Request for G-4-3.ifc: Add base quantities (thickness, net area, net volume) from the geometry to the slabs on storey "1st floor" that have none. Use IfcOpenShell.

First a look at what the model holds.

```python
import ifcopenshell
import ifcopenshell.util.element
import ifcopenshell.util.unit

model = ifcopenshell.open("G-4-3.ifc")
print(model.schema)
for unit_type in ("LENGTHUNIT", "AREAUNIT", "VOLUMEUNIT"):
    print(unit_type, ifcopenshell.util.unit.calculate_unit_scale(model, unit_type))
storey = next(s for s in model.by_type("IfcBuildingStorey") if s.Name == "1st floor")
slabs = [e for e in ifcopenshell.util.element.get_decomposition(storey) if e.is_a("IfcSlab")]
for e in sorted(slabs, key=lambda e: e.id()):
    print(e.id(), e.is_a(), e.Name, list(ifcopenshell.util.element.get_psets(e, qtos_only=True)), sep=" | ")
```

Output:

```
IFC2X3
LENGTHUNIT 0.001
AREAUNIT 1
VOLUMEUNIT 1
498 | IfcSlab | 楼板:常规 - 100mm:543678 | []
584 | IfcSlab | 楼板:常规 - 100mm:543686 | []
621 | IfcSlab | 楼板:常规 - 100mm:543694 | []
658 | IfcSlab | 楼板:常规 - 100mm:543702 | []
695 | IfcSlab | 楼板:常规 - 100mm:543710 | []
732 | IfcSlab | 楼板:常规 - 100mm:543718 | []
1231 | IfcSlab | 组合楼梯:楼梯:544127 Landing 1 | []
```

```python
import ifcopenshell
import ifcopenshell.api.pset
import ifcopenshell.geom
import ifcopenshell.util.element
import ifcopenshell.util.shape
import ifcopenshell.util.unit

model = ifcopenshell.open("G-4-3.ifc")
unit_scale = ifcopenshell.util.unit.calculate_unit_scale(model)
area_scale = ifcopenshell.util.unit.calculate_unit_scale(model, "AREAUNIT")
volume_scale = ifcopenshell.util.unit.calculate_unit_scale(model, "VOLUMEUNIT")
settings = ifcopenshell.geom.settings()

storey = next(s for s in model.by_type("IfcBuildingStorey") if s.Name == "1st floor")
slabs = [e for e in ifcopenshell.util.element.get_decomposition(storey) if e.is_a("IfcSlab")]

for e in sorted(slabs, key=lambda e: e.id()):
    if ifcopenshell.util.element.get_psets(e, qtos_only=True, should_inherit=False):
        continue
    # Geometry comes back in metres, in the element's own axes.
    shape = ifcopenshell.geom.create_shape(settings, e)
    values = {
        "Width": ifcopenshell.util.shape.get_z(shape.geometry) / unit_scale,
        "NetArea": ifcopenshell.util.shape.get_footprint_area(shape.geometry) / area_scale,
        "NetVolume": ifcopenshell.util.shape.get_volume(shape.geometry) / volume_scale,
    }
    qto = ifcopenshell.api.pset.add_qto(model, product=e, name="BaseQuantities")
    ifcopenshell.api.pset.edit_qto(model, qto=qto, properties=values)
    print(e.id(), {k: round(v, 3) for k, v in values.items()})

model.write("G-4-3_updated.ifc")
```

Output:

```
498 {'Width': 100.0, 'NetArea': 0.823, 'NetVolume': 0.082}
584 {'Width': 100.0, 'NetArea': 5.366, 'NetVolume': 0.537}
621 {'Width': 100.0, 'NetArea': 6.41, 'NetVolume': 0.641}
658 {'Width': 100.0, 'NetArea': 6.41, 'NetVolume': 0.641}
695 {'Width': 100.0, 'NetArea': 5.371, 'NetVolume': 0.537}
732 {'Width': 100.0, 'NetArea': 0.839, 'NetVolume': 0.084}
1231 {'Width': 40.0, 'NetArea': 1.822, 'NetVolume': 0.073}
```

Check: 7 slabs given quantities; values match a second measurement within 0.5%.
